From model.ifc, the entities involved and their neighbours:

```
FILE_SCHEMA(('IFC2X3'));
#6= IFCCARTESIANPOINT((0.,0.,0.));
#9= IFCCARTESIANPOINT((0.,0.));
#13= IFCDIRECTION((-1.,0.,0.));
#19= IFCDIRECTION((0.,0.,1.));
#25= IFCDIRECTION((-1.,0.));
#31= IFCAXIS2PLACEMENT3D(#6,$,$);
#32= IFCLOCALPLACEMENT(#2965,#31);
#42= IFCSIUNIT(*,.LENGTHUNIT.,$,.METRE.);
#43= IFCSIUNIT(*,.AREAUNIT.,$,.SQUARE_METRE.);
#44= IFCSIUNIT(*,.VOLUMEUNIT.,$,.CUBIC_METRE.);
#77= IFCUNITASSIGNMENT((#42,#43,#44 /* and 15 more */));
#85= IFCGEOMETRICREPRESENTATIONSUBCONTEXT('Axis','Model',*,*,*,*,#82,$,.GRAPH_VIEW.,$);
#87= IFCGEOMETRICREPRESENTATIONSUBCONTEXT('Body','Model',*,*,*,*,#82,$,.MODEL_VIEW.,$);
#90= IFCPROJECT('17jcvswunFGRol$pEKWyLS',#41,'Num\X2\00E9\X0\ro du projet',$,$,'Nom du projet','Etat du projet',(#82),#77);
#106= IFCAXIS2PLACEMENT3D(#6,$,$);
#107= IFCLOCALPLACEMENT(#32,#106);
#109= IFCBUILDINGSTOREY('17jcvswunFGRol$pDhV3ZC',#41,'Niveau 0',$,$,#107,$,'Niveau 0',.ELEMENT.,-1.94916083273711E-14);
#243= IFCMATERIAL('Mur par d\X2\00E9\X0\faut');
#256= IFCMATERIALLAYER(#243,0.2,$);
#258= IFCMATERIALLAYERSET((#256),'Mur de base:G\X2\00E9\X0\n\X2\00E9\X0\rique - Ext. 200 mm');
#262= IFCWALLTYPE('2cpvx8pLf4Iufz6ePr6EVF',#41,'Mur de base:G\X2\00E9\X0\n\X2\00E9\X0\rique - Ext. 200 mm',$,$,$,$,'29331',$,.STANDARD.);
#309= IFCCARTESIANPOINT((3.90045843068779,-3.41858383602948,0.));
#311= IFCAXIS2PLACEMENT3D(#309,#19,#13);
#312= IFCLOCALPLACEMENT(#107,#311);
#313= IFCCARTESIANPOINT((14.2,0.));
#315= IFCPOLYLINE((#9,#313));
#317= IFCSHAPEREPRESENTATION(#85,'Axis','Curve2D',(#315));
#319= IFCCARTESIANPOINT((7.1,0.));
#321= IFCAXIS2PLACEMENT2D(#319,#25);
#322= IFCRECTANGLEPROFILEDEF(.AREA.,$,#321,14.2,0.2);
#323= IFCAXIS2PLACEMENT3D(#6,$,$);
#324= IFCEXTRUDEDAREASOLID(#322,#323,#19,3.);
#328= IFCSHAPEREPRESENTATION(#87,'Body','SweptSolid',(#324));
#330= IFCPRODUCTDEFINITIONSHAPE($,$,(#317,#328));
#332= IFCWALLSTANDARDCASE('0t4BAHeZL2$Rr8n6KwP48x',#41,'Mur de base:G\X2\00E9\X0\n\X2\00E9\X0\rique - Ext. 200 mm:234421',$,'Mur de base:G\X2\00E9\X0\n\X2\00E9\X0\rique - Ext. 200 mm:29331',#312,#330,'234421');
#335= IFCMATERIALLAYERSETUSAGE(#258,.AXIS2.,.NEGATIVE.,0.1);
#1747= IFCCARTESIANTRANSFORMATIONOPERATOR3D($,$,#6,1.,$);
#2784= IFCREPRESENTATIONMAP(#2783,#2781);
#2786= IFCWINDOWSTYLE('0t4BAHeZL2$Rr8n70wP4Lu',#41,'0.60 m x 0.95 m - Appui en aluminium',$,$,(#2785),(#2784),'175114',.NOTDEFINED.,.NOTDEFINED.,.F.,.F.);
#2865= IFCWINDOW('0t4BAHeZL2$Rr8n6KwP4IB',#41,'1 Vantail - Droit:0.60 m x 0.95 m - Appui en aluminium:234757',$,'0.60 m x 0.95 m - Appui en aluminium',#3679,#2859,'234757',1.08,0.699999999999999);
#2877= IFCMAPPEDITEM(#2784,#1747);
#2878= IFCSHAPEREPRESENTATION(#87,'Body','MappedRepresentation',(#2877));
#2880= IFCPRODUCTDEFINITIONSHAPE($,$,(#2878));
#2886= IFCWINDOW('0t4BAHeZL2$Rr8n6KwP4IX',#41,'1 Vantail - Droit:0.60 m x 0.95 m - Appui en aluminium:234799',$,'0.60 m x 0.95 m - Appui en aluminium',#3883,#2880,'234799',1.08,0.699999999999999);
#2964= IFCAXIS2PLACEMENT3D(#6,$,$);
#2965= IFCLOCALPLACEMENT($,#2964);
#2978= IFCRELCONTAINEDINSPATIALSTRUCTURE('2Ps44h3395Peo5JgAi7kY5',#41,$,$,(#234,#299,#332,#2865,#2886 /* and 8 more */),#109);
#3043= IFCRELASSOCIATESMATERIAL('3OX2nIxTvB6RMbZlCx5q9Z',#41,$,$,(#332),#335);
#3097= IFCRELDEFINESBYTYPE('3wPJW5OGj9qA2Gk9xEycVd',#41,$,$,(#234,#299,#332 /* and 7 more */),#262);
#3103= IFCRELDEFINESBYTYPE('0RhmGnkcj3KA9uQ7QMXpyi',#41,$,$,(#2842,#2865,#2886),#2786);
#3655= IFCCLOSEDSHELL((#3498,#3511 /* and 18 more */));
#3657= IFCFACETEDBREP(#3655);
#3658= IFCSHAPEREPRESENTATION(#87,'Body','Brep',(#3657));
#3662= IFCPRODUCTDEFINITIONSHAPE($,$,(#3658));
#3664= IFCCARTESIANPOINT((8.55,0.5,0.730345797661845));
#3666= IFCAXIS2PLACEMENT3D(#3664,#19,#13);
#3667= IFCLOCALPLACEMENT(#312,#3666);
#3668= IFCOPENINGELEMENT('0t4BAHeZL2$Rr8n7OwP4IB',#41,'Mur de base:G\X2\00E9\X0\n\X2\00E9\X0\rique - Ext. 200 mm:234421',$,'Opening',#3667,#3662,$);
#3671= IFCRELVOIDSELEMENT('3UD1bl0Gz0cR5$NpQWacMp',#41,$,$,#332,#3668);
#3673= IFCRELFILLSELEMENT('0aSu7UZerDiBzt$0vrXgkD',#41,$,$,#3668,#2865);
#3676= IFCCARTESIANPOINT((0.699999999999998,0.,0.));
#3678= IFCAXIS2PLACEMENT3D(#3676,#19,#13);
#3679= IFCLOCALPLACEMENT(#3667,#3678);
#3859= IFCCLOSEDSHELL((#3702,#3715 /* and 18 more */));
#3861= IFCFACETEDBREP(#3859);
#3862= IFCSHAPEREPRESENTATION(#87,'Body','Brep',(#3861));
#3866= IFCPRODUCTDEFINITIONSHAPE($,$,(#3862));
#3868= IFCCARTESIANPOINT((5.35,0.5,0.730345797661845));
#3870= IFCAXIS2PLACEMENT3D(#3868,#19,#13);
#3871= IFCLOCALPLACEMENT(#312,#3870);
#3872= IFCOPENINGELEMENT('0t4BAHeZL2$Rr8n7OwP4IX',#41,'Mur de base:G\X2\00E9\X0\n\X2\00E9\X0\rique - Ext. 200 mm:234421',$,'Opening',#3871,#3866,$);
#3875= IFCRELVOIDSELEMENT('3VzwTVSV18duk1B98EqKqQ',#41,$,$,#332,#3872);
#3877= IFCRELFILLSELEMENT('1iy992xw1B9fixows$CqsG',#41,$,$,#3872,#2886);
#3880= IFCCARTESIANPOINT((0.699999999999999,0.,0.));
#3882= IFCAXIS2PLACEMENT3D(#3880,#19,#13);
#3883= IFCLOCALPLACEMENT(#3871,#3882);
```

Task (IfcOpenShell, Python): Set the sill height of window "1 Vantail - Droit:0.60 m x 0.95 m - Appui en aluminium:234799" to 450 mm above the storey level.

```python
import numpy as np
import ifcopenshell
import ifcopenshell.api.geometry
import ifcopenshell.geom
import ifcopenshell.util.element
import ifcopenshell.util.placement
import ifcopenshell.util.shape
import ifcopenshell.util.unit

model = ifcopenshell.open("model.ifc")
unit_scale = ifcopenshell.util.unit.calculate_unit_scale(model)

window = model.by_guid("0t4BAHeZL2$Rr8n6KwP4IX")
opening = window.FillsVoids[0].RelatingOpeningElement
storey = ifcopenshell.util.element.get_container(window, ifc_class="IfcBuildingStorey")
level = ifcopenshell.util.placement.get_local_placement(storey.ObjectPlacement)[2, 3]

# The opening's origin need not be at the sill, so measure its lowest point.
shape = ifcopenshell.geom.create_shape(ifcopenshell.geom.settings(), opening)
bottom = ifcopenshell.util.shape.get_shape_bottom_elevation(shape, shape.geometry) / unit_scale
dz = level + 0.45 / unit_scale - bottom

shift = np.array([0.0, 0.0, dz])
# The window is placed relative to its opening, so it follows when the opening moves.
matrix = ifcopenshell.util.placement.get_local_placement(opening.ObjectPlacement)
matrix[:3, 3] += shift
ifcopenshell.api.geometry.edit_object_placement(
    model, product=opening, matrix=matrix, is_si=False, should_transform_children=True
)

print(f"moved by {dz * unit_scale:+.3f} m")

model.write("model_edited.ifc")
```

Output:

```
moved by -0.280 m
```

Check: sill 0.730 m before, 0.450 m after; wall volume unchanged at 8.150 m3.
